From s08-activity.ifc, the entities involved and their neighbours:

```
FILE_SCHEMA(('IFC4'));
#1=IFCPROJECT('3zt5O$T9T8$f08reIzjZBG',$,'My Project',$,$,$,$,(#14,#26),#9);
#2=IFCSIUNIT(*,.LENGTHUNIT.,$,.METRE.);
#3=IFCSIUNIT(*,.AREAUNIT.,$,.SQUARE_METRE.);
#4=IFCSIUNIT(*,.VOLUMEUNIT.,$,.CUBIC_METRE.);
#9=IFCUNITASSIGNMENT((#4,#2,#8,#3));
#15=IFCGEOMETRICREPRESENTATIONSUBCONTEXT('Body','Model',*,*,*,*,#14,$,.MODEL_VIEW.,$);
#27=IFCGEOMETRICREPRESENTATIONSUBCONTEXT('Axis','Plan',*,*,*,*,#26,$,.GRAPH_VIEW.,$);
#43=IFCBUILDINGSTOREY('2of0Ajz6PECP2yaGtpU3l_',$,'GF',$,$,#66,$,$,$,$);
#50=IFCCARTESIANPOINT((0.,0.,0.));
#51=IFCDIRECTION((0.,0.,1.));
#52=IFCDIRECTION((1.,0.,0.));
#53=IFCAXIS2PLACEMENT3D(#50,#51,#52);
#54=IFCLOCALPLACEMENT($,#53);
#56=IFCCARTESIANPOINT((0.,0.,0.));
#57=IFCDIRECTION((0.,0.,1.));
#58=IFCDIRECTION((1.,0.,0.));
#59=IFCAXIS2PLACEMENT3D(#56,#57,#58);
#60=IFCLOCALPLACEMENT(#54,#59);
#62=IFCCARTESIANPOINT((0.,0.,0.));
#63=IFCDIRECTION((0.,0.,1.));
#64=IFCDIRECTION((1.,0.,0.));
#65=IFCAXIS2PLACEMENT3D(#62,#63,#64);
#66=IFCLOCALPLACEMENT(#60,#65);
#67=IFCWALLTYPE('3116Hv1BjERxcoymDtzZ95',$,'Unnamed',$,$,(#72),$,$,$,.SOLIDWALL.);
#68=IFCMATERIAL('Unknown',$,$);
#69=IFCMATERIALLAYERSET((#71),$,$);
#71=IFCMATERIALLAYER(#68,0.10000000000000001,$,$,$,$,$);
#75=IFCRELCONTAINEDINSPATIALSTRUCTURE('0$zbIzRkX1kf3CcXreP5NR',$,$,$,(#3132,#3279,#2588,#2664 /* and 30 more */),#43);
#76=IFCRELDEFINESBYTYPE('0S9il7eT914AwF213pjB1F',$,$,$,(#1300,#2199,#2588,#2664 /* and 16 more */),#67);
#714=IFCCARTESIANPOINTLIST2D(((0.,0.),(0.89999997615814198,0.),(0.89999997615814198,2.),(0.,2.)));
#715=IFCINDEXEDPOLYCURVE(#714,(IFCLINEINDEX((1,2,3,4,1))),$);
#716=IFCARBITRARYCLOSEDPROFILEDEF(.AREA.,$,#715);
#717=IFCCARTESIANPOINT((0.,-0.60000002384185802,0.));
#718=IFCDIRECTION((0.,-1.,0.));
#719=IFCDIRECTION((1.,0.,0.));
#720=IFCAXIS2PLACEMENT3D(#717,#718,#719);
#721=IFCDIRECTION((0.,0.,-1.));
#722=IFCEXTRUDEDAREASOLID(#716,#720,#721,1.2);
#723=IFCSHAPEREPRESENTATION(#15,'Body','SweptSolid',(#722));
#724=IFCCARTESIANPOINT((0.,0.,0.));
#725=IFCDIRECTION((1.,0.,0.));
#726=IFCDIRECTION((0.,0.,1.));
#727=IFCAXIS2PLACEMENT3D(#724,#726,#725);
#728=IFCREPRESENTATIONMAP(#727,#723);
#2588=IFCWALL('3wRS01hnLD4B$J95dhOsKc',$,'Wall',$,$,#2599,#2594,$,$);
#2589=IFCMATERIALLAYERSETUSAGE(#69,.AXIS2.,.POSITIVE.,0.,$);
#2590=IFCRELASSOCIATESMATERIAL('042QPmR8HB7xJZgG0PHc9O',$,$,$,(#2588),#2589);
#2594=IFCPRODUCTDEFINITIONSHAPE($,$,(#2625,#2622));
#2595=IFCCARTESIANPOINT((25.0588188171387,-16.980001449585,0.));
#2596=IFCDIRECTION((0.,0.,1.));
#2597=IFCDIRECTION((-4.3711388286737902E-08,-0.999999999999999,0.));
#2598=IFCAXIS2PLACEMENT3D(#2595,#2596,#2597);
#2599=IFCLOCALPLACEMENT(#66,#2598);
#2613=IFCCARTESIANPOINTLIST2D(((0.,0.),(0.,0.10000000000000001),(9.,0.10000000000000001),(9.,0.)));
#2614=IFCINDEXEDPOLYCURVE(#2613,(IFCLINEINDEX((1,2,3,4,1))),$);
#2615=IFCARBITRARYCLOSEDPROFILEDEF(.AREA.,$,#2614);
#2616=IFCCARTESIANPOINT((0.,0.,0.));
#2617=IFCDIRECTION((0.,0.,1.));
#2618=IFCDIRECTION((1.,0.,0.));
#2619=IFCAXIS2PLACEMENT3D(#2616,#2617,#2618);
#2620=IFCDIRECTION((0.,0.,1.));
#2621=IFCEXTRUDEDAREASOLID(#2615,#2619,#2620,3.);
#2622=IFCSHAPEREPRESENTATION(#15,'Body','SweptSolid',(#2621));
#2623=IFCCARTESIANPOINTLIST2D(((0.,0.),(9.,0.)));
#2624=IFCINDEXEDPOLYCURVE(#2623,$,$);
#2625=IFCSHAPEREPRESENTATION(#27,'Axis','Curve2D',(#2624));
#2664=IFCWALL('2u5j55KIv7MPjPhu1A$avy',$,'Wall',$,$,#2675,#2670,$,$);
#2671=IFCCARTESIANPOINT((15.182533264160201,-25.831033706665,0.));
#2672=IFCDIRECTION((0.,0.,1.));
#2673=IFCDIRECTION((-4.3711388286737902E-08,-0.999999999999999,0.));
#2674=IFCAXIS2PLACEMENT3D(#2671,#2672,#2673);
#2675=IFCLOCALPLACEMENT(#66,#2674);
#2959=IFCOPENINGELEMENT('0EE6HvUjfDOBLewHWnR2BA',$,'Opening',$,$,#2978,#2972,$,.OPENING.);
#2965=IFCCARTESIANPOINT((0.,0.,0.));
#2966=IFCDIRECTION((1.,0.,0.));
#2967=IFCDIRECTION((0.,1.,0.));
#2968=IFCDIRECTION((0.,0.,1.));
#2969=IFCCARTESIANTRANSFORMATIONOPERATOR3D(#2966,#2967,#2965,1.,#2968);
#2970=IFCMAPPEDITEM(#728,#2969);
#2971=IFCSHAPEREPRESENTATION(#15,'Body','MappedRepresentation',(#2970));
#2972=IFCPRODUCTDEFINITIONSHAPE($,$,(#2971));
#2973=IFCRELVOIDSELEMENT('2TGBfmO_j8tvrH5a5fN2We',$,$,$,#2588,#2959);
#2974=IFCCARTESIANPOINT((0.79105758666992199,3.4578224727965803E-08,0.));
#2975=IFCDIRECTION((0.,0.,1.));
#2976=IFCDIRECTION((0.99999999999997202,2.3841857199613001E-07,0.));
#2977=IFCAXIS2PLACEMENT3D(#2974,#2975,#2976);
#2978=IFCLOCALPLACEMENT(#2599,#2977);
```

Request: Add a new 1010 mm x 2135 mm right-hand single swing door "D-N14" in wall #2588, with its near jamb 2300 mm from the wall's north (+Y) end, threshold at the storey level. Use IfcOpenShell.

```python
import numpy as np
import ifcopenshell
import ifcopenshell.api.feature
import ifcopenshell.api.geometry
import ifcopenshell.api.root
import ifcopenshell.api.spatial
import ifcopenshell.geom
import ifcopenshell.util.element
import ifcopenshell.util.placement
import ifcopenshell.util.representation
import ifcopenshell.util.shape
import ifcopenshell.util.unit

model = ifcopenshell.open("s08-activity.ifc")
unit_scale = ifcopenshell.util.unit.calculate_unit_scale(model)
settings = ifcopenshell.geom.settings()


def volume(element):
    """Net volume in cubic metres, openings subtracted."""
    shape = ifcopenshell.geom.create_shape(settings, element)
    return ifcopenshell.util.shape.get_volume(shape.geometry)


wall = model.by_guid("3wRS01hnLD4B$J95dhOsKc")
storey = ifcopenshell.util.element.get_container(wall, ifc_class="IfcBuildingStorey")
context = ifcopenshell.util.representation.get_context(model, "Model", "Body", "MODEL_VIEW")
before = volume(wall)

width, height, from_end, sill = 1.01, 2.135, 2.3, 0.0  # metres

# The wall runs along its own X axis, and the end named is its -X end.
wall_shape = ifcopenshell.geom.create_shape(settings, wall)
x, y, z = ifcopenshell.util.shape.get_vertices(wall_shape.geometry).T
start = x.min() + from_end
face, thickness = float(y.min()), float(y.max() - y.min())
wall_matrix = ifcopenshell.util.placement.get_local_placement(wall.ObjectPlacement)
level = ifcopenshell.util.placement.get_local_placement(storey.ObjectPlacement)[2, 3]


def in_wall(x, y):
    """Placement at x, y metres in the wall's axes, at sill height."""
    matrix = wall_matrix.copy()
    matrix[:, 3] = wall_matrix @ np.array([x / unit_scale, y / unit_scale, 0.0, 1.0])
    matrix[2, 3] = level + sill / unit_scale
    return matrix


# Opening: a box that overshoots both wall faces by 50 mm.
opening = ifcopenshell.api.root.create_entity(model, ifc_class="IfcOpeningElement", predefined_type="OPENING")
box = ifcopenshell.api.geometry.add_wall_representation(
    model, context=context, length=width, height=height, thickness=thickness + 0.1
)
ifcopenshell.api.geometry.assign_representation(model, product=opening, representation=box)
ifcopenshell.api.geometry.edit_object_placement(model, product=opening, matrix=in_wall(start, face - 0.05), is_si=False)
ifcopenshell.api.feature.add_feature(model, feature=opening, element=wall)

door = ifcopenshell.api.root.create_entity(model, ifc_class="IfcDoor", name="D-N14", predefined_type="DOOR")
door.OverallWidth, door.OverallHeight = width / unit_scale, height / unit_scale
door.OperationType = "SINGLE_SWING_RIGHT"
body = ifcopenshell.api.geometry.add_door_representation(
    model,
    context=context,
    overall_width=door.OverallWidth,
    overall_height=door.OverallHeight,
    operation_type="SINGLE_SWING_RIGHT",
    lining_properties={"LiningDepth": thickness / unit_scale, "ThresholdDepth": thickness / unit_scale},
)
ifcopenshell.api.geometry.assign_representation(model, product=door, representation=body)
ifcopenshell.api.spatial.assign_container(model, products=[door], relating_structure=storey)
ifcopenshell.api.feature.add_filling(model, opening=opening, element=door)

# The lining spans the wall, so the door starts at the wall face.
ifcopenshell.api.geometry.edit_object_placement(model, product=door, matrix=in_wall(start, face), is_si=False)

after = volume(wall)

print(f"wall volume {before:.3f} -> {after:.3f} m3")

model.write("s08-activity_v2.ifc")
```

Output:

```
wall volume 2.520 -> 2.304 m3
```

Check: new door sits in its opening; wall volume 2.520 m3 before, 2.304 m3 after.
